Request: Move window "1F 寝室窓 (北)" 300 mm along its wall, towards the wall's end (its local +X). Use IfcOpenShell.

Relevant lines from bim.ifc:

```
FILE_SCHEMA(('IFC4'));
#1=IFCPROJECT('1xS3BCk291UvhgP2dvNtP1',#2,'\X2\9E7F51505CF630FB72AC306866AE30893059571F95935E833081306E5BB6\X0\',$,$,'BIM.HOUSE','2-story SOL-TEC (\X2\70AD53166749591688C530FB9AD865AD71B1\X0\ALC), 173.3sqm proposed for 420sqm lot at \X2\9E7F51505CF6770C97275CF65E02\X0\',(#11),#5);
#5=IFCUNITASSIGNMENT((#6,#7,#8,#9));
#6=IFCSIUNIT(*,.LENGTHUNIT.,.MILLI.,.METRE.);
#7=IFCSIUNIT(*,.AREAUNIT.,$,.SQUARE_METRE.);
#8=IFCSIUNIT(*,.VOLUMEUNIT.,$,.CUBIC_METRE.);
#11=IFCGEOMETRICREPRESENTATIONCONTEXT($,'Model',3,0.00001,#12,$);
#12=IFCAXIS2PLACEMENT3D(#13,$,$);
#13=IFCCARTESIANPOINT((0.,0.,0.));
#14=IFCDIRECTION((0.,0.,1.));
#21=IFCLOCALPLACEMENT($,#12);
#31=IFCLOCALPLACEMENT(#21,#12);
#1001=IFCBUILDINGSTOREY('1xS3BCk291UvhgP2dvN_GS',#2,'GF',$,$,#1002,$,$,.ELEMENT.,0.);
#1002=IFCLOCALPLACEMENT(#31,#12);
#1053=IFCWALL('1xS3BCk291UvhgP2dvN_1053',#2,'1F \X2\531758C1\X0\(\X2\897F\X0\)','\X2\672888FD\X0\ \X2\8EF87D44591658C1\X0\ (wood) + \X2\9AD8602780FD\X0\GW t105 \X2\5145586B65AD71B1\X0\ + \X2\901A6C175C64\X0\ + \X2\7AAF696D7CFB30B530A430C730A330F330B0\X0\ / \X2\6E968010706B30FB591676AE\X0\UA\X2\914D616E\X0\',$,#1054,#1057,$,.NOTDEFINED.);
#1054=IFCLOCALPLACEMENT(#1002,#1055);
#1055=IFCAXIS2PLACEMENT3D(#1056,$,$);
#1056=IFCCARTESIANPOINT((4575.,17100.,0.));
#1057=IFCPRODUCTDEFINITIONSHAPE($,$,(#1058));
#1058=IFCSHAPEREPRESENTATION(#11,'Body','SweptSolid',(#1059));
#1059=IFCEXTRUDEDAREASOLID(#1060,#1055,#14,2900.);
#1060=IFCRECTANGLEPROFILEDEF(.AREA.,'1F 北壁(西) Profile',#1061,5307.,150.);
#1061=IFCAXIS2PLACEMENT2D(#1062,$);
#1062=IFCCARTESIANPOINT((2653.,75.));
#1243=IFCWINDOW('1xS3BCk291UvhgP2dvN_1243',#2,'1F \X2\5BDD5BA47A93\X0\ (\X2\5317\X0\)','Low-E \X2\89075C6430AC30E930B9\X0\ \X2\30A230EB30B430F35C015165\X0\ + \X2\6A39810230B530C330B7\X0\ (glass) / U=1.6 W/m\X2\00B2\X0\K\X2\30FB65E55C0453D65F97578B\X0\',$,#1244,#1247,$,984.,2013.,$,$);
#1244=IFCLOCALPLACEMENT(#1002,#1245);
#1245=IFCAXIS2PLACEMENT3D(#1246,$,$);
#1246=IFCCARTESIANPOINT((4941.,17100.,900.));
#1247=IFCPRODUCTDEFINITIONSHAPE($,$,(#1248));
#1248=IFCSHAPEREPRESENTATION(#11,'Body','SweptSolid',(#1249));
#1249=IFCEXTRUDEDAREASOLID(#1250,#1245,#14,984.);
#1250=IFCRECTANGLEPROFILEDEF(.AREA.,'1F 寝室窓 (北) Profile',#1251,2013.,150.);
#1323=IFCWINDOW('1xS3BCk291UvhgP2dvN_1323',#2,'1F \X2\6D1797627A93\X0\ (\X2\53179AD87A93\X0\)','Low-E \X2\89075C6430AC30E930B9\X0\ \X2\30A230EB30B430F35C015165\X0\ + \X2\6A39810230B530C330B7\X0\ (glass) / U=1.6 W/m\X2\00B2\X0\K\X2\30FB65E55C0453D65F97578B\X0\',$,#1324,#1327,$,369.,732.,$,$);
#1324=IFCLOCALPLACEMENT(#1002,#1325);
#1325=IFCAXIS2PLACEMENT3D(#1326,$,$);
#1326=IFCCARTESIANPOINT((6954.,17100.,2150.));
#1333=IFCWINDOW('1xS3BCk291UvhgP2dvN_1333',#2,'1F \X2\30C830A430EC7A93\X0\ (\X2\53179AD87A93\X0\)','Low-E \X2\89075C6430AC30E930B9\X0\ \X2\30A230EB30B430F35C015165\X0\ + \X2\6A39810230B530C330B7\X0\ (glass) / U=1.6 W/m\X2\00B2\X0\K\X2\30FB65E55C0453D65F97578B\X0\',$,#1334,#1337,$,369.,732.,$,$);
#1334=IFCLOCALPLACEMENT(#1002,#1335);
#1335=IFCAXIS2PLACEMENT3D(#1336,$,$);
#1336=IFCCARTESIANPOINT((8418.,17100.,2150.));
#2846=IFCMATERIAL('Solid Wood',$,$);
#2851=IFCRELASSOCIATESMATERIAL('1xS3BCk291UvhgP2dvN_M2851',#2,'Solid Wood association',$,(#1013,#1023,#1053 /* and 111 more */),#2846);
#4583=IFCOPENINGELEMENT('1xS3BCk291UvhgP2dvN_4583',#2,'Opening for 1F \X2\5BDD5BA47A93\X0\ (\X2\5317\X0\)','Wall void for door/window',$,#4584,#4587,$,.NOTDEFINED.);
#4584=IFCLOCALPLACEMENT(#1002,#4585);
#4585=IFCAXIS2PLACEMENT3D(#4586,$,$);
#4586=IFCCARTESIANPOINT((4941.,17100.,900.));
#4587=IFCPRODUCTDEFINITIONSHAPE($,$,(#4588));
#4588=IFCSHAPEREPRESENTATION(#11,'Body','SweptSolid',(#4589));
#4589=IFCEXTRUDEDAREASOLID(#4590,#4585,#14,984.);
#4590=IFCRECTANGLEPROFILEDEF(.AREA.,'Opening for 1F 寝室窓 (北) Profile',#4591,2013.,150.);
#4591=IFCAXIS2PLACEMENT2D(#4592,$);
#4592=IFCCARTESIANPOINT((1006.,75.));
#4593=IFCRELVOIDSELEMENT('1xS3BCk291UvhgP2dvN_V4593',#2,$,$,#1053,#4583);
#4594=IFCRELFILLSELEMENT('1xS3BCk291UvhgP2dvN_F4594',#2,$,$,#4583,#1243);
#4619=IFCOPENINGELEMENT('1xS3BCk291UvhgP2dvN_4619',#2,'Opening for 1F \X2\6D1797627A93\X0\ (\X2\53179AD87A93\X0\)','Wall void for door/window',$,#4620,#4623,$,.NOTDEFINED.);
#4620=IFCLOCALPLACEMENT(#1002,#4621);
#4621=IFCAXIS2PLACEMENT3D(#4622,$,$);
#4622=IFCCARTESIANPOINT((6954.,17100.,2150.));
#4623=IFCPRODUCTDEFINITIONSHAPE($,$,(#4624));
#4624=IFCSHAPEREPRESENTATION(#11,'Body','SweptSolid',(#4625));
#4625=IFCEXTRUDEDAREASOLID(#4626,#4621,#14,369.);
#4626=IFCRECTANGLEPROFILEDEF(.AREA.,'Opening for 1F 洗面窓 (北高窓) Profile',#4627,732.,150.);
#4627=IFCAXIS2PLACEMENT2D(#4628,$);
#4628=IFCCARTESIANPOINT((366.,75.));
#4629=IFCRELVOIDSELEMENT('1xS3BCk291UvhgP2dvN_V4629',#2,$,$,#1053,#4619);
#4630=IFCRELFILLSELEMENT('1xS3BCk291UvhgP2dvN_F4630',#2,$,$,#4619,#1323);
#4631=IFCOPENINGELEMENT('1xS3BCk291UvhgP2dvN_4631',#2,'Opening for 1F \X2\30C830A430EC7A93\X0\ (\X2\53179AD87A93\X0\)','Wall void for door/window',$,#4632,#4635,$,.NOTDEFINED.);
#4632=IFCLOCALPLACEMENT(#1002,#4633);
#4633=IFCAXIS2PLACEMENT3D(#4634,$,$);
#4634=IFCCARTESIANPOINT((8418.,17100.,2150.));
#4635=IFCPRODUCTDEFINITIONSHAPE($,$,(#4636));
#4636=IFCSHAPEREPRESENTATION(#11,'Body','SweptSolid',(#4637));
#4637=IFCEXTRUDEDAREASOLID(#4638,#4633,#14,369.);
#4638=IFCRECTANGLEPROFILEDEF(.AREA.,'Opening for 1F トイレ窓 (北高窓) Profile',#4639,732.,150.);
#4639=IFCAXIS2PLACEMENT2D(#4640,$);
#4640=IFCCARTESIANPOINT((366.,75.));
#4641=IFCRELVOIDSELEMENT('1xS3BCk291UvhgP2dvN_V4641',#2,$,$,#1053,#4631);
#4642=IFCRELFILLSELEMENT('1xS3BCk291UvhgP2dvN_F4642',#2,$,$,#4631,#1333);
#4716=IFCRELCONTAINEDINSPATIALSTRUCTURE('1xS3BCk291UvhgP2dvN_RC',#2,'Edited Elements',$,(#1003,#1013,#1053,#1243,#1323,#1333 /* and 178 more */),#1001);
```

```python
import ifcopenshell
import ifcopenshell.api.geometry
import ifcopenshell.util.placement

model = ifcopenshell.open("bim.ifc")

window = model.by_id(1243)
opening = window.FillsVoids[0].RelatingOpeningElement
wall = opening.VoidsElements[0].RelatingBuildingElement

wall_matrix = ifcopenshell.util.placement.get_local_placement(wall.ObjectPlacement)
shift = wall_matrix[:3, 0] * 300.0
before = ifcopenshell.util.placement.get_local_placement(window.ObjectPlacement)[:3, 3].copy()

# The window is not placed relative to its opening, so move both.
for product in (opening, window):
    matrix = ifcopenshell.util.placement.get_local_placement(product.ObjectPlacement)
    matrix[:3, 3] += shift
    ifcopenshell.api.geometry.edit_object_placement(model, product=product, matrix=matrix, is_si=False)

after = ifcopenshell.util.placement.get_local_placement(window.ObjectPlacement)[:3, 3]
print("window moved by", (after - before).round(3) + 0.0)

model.write("bim_rev.ifc")
```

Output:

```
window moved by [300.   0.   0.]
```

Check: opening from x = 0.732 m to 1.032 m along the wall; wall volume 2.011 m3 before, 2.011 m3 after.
